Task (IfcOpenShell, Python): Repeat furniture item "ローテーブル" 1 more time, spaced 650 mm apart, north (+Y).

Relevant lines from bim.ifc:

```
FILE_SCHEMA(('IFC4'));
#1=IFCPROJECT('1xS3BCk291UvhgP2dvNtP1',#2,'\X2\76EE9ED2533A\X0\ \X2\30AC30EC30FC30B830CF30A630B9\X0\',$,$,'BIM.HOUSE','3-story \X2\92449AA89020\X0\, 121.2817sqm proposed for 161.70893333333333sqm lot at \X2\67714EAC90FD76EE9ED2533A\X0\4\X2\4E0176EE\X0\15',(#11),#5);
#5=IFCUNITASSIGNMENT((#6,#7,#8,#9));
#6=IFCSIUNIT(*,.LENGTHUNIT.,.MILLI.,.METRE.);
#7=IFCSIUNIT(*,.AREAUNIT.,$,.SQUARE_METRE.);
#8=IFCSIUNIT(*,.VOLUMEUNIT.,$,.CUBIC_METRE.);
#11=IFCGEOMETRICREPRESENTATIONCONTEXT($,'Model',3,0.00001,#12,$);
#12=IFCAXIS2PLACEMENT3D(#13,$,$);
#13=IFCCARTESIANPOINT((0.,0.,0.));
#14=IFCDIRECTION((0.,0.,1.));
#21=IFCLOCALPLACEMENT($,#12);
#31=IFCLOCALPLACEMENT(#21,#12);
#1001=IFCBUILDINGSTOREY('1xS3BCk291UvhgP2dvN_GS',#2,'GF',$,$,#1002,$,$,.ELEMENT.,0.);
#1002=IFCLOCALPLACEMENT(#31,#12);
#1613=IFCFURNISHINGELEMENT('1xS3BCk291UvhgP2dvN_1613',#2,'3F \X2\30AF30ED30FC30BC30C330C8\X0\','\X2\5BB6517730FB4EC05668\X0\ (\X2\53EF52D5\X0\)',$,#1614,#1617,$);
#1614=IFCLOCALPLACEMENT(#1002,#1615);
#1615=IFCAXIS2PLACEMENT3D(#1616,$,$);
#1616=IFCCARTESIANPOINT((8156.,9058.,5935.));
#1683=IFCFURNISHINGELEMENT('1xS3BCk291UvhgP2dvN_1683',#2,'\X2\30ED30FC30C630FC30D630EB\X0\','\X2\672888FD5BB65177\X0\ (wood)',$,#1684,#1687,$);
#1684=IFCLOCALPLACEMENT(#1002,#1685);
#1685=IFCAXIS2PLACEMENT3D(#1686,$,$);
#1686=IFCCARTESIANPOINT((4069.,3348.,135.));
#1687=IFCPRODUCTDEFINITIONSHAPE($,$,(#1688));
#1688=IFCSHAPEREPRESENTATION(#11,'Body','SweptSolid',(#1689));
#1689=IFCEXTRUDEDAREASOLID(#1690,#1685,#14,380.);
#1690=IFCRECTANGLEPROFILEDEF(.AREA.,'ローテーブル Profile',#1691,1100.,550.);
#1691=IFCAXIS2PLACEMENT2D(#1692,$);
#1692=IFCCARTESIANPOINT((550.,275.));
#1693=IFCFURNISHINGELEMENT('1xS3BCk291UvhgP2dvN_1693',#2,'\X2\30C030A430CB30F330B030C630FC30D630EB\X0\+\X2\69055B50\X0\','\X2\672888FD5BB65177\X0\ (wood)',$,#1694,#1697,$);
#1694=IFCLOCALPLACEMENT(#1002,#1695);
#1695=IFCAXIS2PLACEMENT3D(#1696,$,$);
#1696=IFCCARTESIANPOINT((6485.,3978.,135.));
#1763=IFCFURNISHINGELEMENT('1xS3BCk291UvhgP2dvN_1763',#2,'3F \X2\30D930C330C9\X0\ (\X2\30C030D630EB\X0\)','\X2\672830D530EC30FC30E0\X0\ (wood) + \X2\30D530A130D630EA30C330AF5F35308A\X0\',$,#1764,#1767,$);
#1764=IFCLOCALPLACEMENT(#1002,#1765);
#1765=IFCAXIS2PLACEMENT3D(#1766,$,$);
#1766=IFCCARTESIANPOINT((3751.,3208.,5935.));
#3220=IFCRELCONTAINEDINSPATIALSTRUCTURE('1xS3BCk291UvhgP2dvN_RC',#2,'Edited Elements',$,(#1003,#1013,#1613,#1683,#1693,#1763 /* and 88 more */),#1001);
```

```python
import numpy as np
import ifcopenshell
import ifcopenshell.api.geometry
import ifcopenshell.api.root
import ifcopenshell.util.element
import ifcopenshell.util.placement
import ifcopenshell.util.unit

model = ifcopenshell.open("bim.ifc")
unit_scale = ifcopenshell.util.unit.calculate_unit_scale(model)


def reuse_history(source, copy):
    """copy_class also copies each property set's owner history, people and application; keep the originals."""
    for rel in copy.IsDefinedBy:
        if rel.is_a("IfcRelDefinesByProperties") and (history := rel.RelatingPropertyDefinition.OwnerHistory):
            rel.RelatingPropertyDefinition.OwnerHistory = source.OwnerHistory
            ifcopenshell.util.element.remove_deep2(model, history)


source = model.by_guid("1xS3BCk291UvhgP2dvN_1683")
base = ifcopenshell.util.placement.get_local_placement(source.ObjectPlacement)
step = np.array([0.0, 1.0, 0.0]) * 0.65 / unit_scale

for i in range(1, 2):
    copy = ifcopenshell.api.root.copy_class(model, product=source)
    copy.Representation = ifcopenshell.util.element.copy_deep(
        model, source.Representation, exclude=["IfcGeometricRepresentationContext", "IfcRepresentationMap"]
    )
    reuse_history(source, copy)
    matrix = base.copy()
    matrix[:3, 3] += i * step
    print("added at", matrix[:3, 3].round(3) + 0.0)
    ifcopenshell.api.geometry.edit_object_placement(model, product=copy, matrix=matrix, is_si=False)

model.write("bim_v2.ifc")
```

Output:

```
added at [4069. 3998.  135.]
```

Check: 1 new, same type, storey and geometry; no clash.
